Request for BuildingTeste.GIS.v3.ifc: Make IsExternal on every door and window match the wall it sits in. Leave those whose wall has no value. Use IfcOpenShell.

First a look at what the model holds.

```python
import ifcopenshell
import ifcopenshell.util.element

model = ifcopenshell.open("BuildingTeste.GIS.v3.ifc")
print(model.schema)
seen = {}
for e in model.by_type("IfcDoor") + model.by_type("IfcWindow"):
    if not e.FillsVoids:
        continue
    host = e.FillsVoids[0].RelatingOpeningElement.VoidsElements[0].RelatingBuildingElement
    own = ifcopenshell.util.element.get_pset(e, f"Pset_{e.is_a()[3:].removesuffix('StandardCase')}Common", "IsExternal")
    wall = ifcopenshell.util.element.get_pset(host, "Pset_WallCommon", "IsExternal")
    seen[e.is_a(), own, wall] = seen.get((e.is_a(), own, wall), 0) + 1
for (cls, own, wall), count in sorted(seen.items(), key=str):
    print(count, cls, "IsExternal:", own, "| host wall:", wall)
```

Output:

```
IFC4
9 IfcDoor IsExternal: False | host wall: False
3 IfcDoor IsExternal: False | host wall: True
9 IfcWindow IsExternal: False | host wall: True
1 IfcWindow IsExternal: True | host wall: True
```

```python
import ifcopenshell
import ifcopenshell.api.pset
import ifcopenshell.util.element

model = ifcopenshell.open("BuildingTeste.GIS.v3.ifc")

count = 0
for ifc_class, pset_name in (("IfcDoor", "Pset_DoorCommon"), ("IfcWindow", "Pset_WindowCommon")):
    for e in model.by_type(ifc_class):
        if not e.FillsVoids:
            continue
        host = e.FillsVoids[0].RelatingOpeningElement.VoidsElements[0].RelatingBuildingElement
        external = ifcopenshell.util.element.get_pset(host, "Pset_WallCommon", "IsExternal")
        if external is None or ifcopenshell.util.element.get_pset(e, pset_name, "IsExternal") == external:
            continue
        pset = ifcopenshell.api.pset.add_pset(model, product=e, name=pset_name)
        ifcopenshell.api.pset.edit_pset(model, pset=pset, properties={"IsExternal": external})
        count += 1

print(count, "updated")

model.write("BuildingTeste.GIS.v3_updated.ifc")
```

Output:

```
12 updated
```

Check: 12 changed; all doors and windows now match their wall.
